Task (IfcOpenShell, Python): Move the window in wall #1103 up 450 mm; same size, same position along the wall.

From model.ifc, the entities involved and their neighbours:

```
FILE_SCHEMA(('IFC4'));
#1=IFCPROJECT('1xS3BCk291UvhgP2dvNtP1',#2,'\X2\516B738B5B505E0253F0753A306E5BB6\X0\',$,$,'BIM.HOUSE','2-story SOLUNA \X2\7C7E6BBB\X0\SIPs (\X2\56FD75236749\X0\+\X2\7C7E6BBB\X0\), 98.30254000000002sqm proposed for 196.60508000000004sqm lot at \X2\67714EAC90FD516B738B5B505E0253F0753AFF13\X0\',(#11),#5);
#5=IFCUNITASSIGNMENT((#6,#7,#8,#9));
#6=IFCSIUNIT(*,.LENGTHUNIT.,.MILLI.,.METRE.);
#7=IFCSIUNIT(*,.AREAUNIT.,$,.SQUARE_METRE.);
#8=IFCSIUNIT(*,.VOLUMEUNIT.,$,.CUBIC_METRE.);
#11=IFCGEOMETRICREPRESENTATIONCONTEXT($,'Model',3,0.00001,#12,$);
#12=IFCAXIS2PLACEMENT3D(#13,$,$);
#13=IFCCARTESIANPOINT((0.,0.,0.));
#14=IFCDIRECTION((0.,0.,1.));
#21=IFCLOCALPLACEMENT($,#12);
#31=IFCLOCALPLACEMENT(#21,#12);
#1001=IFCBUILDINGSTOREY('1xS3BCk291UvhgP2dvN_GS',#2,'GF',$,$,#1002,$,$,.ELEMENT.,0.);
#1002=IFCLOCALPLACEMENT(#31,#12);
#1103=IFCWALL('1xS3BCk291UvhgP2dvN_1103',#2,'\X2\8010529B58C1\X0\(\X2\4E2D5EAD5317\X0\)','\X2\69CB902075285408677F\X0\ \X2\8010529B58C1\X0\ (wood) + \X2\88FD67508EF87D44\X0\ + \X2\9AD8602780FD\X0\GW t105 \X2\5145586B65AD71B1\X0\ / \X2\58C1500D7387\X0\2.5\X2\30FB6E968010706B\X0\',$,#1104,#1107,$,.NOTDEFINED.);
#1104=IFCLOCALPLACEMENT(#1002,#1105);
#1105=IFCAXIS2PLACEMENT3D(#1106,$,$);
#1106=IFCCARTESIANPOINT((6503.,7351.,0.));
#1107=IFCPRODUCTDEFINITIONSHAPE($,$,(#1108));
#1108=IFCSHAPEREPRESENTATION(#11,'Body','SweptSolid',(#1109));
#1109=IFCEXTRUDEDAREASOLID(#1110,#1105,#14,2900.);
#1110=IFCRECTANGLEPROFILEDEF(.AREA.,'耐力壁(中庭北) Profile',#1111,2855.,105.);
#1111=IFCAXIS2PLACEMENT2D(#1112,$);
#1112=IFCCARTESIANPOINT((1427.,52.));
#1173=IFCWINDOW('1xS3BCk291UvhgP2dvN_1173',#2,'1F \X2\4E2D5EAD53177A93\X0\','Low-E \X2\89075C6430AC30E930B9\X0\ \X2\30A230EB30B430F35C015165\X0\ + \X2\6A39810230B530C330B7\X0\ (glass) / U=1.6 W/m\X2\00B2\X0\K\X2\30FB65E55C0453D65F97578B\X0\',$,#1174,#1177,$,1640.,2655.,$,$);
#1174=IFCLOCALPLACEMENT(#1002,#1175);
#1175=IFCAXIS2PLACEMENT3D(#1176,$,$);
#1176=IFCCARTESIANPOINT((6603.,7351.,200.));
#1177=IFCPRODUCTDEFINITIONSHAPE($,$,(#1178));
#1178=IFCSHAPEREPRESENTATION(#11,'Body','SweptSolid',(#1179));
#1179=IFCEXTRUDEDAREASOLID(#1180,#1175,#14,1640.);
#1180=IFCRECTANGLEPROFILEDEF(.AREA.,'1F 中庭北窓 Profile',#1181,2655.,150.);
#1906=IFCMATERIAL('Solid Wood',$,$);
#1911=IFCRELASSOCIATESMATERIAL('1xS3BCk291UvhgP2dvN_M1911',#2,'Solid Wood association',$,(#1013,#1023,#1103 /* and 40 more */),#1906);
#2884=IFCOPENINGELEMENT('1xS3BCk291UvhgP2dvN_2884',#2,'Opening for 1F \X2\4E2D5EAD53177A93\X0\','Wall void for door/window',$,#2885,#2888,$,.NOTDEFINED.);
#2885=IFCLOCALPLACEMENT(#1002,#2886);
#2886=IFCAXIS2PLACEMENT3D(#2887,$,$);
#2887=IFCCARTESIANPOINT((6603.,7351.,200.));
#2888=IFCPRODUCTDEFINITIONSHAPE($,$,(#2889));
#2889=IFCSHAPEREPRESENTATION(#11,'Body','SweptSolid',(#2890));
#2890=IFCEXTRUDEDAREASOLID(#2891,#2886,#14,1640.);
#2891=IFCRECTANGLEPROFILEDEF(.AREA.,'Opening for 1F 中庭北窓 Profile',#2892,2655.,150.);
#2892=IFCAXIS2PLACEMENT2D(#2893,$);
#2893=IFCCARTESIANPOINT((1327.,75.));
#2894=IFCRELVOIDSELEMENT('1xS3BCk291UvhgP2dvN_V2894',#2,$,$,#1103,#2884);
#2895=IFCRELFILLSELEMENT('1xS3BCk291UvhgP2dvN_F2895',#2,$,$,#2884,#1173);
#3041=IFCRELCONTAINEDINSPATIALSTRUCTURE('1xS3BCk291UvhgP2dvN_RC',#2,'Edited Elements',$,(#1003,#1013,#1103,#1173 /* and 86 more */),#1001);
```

```python
import numpy as np
import ifcopenshell
import ifcopenshell.api.geometry
import ifcopenshell.util.placement
import ifcopenshell.util.unit

model = ifcopenshell.open("model.ifc")
unit_scale = ifcopenshell.util.unit.calculate_unit_scale(model)

window = model.by_guid("1xS3BCk291UvhgP2dvN_1173")
opening = window.FillsVoids[0].RelatingOpeningElement
dz = 450.0

shift = np.array([0.0, 0.0, dz])
# The window is not placed relative to its opening, so move both.
for product in (opening, window):
    matrix = ifcopenshell.util.placement.get_local_placement(product.ObjectPlacement)
    matrix[:3, 3] += shift
    ifcopenshell.api.geometry.edit_object_placement(model, product=product, matrix=matrix, is_si=False)

print(f"moved by {dz * unit_scale:+.3f} m")

model.write("model_rev.ifc")
```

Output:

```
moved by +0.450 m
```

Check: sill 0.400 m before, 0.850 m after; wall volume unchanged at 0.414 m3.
